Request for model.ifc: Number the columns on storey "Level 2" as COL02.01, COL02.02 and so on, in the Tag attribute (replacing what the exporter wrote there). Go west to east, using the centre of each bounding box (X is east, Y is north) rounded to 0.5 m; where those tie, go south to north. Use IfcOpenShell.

First a look at what the model holds.

```python
import ifcopenshell
import ifcopenshell.util.element
import ifcopenshell.util.placement

model = ifcopenshell.open("model.ifc")
print(model.schema)
storey = next(s for s in model.by_type("IfcBuildingStorey") if s.Name == "Level 2")
columns = [e for e in ifcopenshell.util.element.get_decomposition(storey) if e.is_a("IfcColumn")]
for e in sorted(columns, key=lambda e: e.id()):
    origin = ifcopenshell.util.placement.get_local_placement(e.ObjectPlacement)[:3, 3]
    print(e.id(), e.Tag, e.Name, origin.round(2) + 0.0, sep=" | ")
```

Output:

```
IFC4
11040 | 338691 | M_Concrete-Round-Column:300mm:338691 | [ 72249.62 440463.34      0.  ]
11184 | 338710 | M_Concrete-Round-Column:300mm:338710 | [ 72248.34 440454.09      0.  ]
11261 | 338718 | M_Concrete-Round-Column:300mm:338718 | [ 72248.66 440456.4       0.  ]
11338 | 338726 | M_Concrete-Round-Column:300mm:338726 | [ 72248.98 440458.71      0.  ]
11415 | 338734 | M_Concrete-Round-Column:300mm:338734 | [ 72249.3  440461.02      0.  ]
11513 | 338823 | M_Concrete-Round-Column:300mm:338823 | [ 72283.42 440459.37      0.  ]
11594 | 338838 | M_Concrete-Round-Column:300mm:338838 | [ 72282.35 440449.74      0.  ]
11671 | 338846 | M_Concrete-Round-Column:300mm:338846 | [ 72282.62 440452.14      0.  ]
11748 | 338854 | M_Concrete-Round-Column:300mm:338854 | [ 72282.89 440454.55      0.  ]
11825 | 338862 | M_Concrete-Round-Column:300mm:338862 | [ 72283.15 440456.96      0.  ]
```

```python
import ifcopenshell
import ifcopenshell.geom
import ifcopenshell.util.element
import ifcopenshell.util.shape

model = ifcopenshell.open("model.ifc")
settings = ifcopenshell.geom.settings()
settings.set("use-world-coords", True)


def centre(element):
    shape = ifcopenshell.geom.create_shape(settings, element)
    return ifcopenshell.util.shape.get_bbox_centroid(shape.geometry)


storey = next(s for s in model.by_type("IfcBuildingStorey") if s.Name == "Level 2")
columns = [e for e in ifcopenshell.util.element.get_decomposition(storey) if e.is_a("IfcColumn")]

# Insertion points can sit at a corner or the storey origin, so sort by the geometry (in metres).
centres = {e: centre(e) for e in columns}
columns.sort(key=lambda e: (round(centres[e][0] / 0.5), centres[e][1]))

for i, e in enumerate(columns, start=1):
    number = f"COL02.{i:02d}"
    e.Tag = number
    print(e.id(), number)

model.write("model_updated.ifc")
```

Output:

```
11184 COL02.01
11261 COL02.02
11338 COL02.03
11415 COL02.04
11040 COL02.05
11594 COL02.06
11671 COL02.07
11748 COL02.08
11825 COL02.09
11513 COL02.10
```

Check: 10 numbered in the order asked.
